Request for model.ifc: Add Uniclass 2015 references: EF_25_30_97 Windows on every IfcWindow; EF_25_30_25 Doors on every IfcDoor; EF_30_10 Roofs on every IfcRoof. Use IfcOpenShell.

First a look at what the model holds.

```python
import ifcopenshell

model = ifcopenshell.open("model.ifc")
print(model.schema)
print("classifications:", [c.Name for c in model.by_type("IfcClassification")])
for ifc_class in ("IfcDoor", "IfcRoof", "IfcStair", "IfcWall", "IfcWindow"):
    print(ifc_class, len(model.by_type(ifc_class)))
```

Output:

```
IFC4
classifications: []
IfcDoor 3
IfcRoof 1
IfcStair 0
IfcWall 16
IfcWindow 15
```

```python
import ifcopenshell
import ifcopenshell.api.classification

model = ifcopenshell.open("model.ifc")

system = ifcopenshell.api.classification.add_classification(model, classification="Uniclass 2015")

codes = {
    "IfcWindow": ("EF_25_30_97", "Windows"),
    "IfcDoor": ("EF_25_30_25", "Doors"),
    "IfcRoof": ("EF_30_10", "Roofs"),
}
for ifc_class, (code, name) in codes.items():
    products = model.by_type(ifc_class)
    ifcopenshell.api.classification.add_reference(
        model, products=products, classification=system, identification=code, name=name
    )
    print(code, len(products))

model.write("model-out.ifc")
```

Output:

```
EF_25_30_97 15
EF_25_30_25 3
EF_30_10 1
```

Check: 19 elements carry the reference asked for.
